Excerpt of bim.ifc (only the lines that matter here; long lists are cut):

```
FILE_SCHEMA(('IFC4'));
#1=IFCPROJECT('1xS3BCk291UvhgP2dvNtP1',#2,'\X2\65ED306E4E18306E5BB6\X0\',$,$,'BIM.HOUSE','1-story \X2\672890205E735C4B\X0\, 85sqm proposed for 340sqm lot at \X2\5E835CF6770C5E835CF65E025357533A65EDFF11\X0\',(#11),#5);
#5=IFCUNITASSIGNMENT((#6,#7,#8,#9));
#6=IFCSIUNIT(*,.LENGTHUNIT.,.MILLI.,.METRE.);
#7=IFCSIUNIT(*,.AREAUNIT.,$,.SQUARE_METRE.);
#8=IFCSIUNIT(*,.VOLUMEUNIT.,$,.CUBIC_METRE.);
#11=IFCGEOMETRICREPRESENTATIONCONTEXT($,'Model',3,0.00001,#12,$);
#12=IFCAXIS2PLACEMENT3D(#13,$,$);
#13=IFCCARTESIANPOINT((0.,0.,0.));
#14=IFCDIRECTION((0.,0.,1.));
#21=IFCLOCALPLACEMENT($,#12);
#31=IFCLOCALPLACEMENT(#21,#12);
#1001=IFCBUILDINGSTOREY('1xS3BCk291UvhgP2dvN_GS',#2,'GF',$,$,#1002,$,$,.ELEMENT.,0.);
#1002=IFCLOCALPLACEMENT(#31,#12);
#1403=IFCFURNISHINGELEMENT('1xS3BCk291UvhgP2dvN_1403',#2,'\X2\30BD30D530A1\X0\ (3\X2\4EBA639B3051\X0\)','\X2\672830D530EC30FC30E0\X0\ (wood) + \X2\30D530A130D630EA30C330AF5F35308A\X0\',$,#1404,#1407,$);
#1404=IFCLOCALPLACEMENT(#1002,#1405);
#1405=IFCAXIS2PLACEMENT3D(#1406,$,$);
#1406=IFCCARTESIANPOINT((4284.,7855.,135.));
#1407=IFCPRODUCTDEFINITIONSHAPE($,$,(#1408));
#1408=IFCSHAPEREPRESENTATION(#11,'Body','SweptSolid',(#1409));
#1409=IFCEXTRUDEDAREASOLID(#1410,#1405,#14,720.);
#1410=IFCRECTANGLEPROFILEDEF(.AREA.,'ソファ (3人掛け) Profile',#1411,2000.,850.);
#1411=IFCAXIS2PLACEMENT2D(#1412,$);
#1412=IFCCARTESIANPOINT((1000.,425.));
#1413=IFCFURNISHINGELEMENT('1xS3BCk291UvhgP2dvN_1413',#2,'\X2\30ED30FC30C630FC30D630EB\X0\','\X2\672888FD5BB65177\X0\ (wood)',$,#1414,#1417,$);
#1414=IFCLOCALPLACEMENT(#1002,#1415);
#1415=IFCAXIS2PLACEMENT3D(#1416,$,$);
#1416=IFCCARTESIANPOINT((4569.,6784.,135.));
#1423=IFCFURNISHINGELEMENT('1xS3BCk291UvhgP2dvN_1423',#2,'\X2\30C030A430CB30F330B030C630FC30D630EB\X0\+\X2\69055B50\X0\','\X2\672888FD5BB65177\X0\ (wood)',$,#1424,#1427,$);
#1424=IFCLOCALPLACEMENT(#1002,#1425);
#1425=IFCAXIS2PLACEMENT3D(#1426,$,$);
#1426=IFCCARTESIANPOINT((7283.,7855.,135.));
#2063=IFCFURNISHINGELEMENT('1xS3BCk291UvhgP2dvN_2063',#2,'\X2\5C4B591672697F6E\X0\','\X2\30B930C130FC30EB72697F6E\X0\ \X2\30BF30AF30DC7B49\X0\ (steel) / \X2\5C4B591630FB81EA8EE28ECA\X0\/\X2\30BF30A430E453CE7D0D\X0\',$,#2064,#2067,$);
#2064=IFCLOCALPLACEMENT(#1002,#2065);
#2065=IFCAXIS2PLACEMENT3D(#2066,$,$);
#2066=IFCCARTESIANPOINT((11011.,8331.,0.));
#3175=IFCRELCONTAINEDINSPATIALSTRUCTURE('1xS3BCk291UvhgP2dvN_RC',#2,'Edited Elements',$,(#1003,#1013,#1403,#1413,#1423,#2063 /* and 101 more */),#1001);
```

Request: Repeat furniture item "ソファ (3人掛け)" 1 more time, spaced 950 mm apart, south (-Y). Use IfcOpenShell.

```python
import numpy as np
import ifcopenshell
import ifcopenshell.api.geometry
import ifcopenshell.api.root
import ifcopenshell.util.element
import ifcopenshell.util.placement

model = ifcopenshell.open("bim.ifc")


def reuse_history(source, copy):
    """copy_class also copies each property set's owner history, people and application; keep the originals."""
    for rel in copy.IsDefinedBy:
        if rel.is_a("IfcRelDefinesByProperties") and (history := rel.RelatingPropertyDefinition.OwnerHistory):
            rel.RelatingPropertyDefinition.OwnerHistory = source.OwnerHistory
            ifcopenshell.util.element.remove_deep2(model, history)


source = model.by_id(1403)
base = ifcopenshell.util.placement.get_local_placement(source.ObjectPlacement)
step = np.array([0.0, -1.0, 0.0]) * 950.0

for i in range(1, 2):
    copy = ifcopenshell.api.root.copy_class(model, product=source)
    copy.Representation = ifcopenshell.util.element.copy_deep(
        model, source.Representation, exclude=["IfcGeometricRepresentationContext", "IfcRepresentationMap"]
    )
    reuse_history(source, copy)
    matrix = base.copy()
    matrix[:3, 3] += i * step
    print("added at", matrix[:3, 3].round(3) + 0.0)
    ifcopenshell.api.geometry.edit_object_placement(model, product=copy, matrix=matrix, is_si=False)

model.write("bim_rev.ifc")
```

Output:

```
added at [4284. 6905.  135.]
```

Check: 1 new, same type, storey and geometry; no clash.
